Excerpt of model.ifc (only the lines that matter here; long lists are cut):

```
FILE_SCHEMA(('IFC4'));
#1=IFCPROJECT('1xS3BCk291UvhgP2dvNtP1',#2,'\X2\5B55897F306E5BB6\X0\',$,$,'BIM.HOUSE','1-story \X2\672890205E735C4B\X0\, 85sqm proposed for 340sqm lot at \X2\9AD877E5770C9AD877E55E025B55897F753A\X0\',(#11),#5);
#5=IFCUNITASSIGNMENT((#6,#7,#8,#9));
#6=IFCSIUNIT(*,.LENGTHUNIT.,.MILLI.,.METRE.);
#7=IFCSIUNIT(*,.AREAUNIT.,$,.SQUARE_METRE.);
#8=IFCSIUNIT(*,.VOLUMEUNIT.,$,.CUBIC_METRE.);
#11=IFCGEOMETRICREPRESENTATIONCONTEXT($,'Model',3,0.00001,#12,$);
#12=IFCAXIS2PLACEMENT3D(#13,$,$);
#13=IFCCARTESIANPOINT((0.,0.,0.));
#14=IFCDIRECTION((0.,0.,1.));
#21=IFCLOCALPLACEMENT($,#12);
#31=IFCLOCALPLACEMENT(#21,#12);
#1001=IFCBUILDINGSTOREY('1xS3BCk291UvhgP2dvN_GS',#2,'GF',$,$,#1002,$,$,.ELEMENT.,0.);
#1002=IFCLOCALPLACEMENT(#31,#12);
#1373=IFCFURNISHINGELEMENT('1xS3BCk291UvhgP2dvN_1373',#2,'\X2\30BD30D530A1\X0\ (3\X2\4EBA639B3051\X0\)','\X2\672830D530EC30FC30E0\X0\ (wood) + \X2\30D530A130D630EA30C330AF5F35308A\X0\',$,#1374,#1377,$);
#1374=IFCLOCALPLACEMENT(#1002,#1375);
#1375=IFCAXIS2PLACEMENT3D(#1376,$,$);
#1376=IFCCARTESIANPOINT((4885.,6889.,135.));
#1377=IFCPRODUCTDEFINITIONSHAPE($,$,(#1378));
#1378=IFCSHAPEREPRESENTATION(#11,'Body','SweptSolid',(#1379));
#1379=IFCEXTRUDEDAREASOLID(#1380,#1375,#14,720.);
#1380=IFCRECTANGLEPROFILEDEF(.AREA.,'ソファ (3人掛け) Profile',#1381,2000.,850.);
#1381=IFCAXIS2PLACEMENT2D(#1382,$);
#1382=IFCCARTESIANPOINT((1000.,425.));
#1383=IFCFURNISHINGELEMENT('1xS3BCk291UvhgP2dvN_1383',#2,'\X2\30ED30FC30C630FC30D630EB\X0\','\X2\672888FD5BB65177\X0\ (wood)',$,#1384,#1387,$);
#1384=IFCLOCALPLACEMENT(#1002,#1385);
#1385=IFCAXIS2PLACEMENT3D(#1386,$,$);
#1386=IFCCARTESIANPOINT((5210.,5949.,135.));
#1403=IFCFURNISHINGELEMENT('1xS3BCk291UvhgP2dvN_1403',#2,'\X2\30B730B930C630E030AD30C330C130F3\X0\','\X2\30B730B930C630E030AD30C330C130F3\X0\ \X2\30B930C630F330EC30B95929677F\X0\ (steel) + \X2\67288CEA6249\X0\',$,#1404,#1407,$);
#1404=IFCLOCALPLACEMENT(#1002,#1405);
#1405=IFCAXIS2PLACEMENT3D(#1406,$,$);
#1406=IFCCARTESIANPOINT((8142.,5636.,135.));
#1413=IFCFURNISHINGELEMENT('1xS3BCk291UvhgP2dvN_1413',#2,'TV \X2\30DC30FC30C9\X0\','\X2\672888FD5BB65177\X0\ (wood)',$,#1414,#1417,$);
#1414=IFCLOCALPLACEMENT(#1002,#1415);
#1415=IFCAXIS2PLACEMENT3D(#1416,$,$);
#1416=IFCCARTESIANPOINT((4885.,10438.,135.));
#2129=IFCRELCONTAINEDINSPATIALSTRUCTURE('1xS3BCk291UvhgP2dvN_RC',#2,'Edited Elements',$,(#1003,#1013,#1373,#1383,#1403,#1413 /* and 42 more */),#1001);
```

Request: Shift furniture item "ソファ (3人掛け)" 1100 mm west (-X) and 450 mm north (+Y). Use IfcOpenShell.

```python
import ifcopenshell
import ifcopenshell.api.geometry
import ifcopenshell.util.placement
import ifcopenshell.util.unit

model = ifcopenshell.open("model.ifc")
unit_scale = ifcopenshell.util.unit.calculate_unit_scale(model)

item = model.by_guid("1xS3BCk291UvhgP2dvN_1373")
matrix = ifcopenshell.util.placement.get_local_placement(item.ObjectPlacement)
matrix[0, 3] -= 1.1 / unit_scale
matrix[1, 3] += 0.45 / unit_scale
ifcopenshell.api.geometry.edit_object_placement(model, product=item, matrix=matrix, is_si=False)

print(ifcopenshell.util.placement.get_local_placement(item.ObjectPlacement).round(3) + 0.0)

model.write("model_updated.ifc")
```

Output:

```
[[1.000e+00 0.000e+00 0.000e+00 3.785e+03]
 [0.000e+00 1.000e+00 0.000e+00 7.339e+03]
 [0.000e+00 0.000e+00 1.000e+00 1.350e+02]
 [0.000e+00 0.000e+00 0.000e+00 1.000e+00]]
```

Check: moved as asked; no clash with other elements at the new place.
